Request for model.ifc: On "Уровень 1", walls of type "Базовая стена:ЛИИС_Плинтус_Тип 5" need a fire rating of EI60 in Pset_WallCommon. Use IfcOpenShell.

First a look at what the model holds.

```python
import ifcopenshell
import ifcopenshell.util.element

model = ifcopenshell.open("model.ifc")
print(model.schema)
storey = next(s for s in model.by_type("IfcBuildingStorey") if s.Name == "Уровень 1")
walls = [e for e in ifcopenshell.util.element.get_decomposition(storey) if e.is_a("IfcWall")]
seen = {}
for e in walls:
    element_type = ifcopenshell.util.element.get_type(e)
    key = (element_type.Name if element_type != e and element_type else None, ifcopenshell.util.element.get_pset(e, "Pset_WallCommon", "FireRating"))
    seen[key] = seen.get(key, 0) + 1
for (name, value), count in sorted(seen.items(), key=str):
    print(count, "x", name, "|", value)
```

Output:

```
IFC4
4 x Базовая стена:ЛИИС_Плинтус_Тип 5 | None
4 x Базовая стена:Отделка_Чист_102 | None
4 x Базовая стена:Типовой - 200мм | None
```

```python
import ifcopenshell
import ifcopenshell.api.pset
import ifcopenshell.util.element

model = ifcopenshell.open("model.ifc")

storey = next(s for s in model.by_type("IfcBuildingStorey") if s.Name == "Уровень 1")
walls = [e for e in ifcopenshell.util.element.get_decomposition(storey) if e.is_a("IfcWall")]

count = 0
for e in walls:
    element_type = ifcopenshell.util.element.get_type(e)
    if element_type in (None, e) or element_type.Name != "Базовая стена:ЛИИС_Плинтус_Тип 5":
        continue
    # add_pset returns the element's existing set when there is one.
    pset = ifcopenshell.api.pset.add_pset(model, product=e, name="Pset_WallCommon")
    ifcopenshell.api.pset.edit_pset(model, pset=pset, properties={"FireRating": "EI60"})
    count += 1

print(count, "walls updated")

model.write("model_edited.ifc")
```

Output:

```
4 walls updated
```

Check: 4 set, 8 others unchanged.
